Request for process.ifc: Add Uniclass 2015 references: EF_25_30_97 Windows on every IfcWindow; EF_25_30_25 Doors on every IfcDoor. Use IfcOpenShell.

First a look at what the model holds.

```python
import ifcopenshell

model = ifcopenshell.open("process.ifc")
print(model.schema)
print("classifications:", [c.Name for c in model.by_type("IfcClassification")])
for ifc_class in ("IfcDoor", "IfcRoof", "IfcStair", "IfcWall", "IfcWindow"):
    print(ifc_class, len(model.by_type(ifc_class)))
```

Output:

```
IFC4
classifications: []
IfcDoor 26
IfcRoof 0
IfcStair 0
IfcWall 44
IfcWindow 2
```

```python
import ifcopenshell
import ifcopenshell.api.classification

model = ifcopenshell.open("process.ifc")

system = ifcopenshell.api.classification.add_classification(model, classification="Uniclass 2015")

codes = {
    "IfcWindow": ("EF_25_30_97", "Windows"),
    "IfcDoor": ("EF_25_30_25", "Doors"),
}
for ifc_class, (code, name) in codes.items():
    products = model.by_type(ifc_class)
    ifcopenshell.api.classification.add_reference(
        model, products=products, classification=system, identification=code, name=name
    )
    print(code, len(products))

model.write("process_updated.ifc")
```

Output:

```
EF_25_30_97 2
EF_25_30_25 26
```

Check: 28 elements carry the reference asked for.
